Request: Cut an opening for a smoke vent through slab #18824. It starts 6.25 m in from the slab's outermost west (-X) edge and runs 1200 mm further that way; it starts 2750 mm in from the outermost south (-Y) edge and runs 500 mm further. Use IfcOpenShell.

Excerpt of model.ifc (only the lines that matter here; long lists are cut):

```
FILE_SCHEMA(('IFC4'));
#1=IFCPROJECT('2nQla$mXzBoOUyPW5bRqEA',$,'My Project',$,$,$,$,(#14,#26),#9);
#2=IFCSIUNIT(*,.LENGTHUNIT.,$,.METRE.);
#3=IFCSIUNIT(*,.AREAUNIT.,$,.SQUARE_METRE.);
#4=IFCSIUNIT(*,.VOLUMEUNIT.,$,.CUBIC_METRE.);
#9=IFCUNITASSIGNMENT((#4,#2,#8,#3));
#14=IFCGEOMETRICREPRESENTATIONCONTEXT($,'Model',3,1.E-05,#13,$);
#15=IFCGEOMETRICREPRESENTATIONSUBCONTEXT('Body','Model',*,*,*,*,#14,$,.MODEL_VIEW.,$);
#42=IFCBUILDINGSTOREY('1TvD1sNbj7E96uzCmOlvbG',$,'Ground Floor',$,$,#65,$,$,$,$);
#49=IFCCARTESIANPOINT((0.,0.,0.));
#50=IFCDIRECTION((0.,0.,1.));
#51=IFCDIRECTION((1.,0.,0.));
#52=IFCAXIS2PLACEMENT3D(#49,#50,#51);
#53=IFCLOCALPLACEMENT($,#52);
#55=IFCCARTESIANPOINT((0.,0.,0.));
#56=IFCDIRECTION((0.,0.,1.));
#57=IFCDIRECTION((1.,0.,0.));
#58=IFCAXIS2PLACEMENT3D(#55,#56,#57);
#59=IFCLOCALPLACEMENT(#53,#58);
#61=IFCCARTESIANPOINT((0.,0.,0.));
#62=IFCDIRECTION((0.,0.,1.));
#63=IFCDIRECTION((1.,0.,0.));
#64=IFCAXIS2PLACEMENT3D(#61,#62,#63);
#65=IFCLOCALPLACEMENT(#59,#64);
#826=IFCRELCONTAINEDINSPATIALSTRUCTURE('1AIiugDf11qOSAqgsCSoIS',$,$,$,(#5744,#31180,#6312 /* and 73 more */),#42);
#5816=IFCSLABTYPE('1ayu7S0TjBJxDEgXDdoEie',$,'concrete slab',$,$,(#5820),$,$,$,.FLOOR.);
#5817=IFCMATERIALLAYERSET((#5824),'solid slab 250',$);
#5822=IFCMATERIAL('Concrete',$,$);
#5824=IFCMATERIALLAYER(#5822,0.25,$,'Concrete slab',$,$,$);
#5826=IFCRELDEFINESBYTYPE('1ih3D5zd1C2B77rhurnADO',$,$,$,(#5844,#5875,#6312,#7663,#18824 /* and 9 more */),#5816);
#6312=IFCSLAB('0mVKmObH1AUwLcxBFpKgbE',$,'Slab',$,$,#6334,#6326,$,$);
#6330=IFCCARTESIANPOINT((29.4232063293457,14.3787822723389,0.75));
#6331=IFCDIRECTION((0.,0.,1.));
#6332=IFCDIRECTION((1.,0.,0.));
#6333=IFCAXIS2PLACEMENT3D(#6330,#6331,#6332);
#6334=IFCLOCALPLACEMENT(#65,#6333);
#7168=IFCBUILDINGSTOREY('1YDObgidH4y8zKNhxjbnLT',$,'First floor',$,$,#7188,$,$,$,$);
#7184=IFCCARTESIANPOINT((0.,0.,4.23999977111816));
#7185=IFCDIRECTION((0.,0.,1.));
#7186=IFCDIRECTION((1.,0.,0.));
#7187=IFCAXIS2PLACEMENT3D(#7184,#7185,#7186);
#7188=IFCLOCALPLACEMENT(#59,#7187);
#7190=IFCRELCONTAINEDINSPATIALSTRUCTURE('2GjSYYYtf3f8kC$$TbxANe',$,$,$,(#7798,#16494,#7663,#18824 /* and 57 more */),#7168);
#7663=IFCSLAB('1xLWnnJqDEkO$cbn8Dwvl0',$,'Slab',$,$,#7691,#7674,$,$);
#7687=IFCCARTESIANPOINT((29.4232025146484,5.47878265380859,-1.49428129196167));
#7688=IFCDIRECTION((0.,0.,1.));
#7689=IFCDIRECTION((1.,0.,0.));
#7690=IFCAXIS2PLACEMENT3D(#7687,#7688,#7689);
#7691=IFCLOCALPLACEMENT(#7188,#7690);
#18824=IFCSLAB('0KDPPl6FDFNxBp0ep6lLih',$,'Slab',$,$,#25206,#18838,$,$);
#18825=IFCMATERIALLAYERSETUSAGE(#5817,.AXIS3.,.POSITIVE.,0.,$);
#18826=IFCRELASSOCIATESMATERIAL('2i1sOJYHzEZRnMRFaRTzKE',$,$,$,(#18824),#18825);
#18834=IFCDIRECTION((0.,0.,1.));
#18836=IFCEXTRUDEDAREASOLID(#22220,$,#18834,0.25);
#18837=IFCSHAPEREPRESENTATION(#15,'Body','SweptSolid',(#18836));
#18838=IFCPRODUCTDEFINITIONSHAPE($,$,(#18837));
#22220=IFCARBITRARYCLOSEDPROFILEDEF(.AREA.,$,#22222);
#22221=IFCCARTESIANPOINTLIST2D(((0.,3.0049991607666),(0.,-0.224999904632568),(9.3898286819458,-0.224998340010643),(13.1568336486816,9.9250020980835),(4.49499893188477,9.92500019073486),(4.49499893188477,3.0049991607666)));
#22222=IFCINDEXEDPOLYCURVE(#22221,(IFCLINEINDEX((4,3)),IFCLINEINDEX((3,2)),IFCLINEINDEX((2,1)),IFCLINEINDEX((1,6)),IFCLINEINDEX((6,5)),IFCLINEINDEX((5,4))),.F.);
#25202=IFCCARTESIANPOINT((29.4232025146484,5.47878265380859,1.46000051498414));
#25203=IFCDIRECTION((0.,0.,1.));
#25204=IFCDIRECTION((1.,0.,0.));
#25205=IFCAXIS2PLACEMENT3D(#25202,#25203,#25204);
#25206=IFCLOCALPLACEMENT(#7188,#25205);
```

```python
import numpy as np
import ifcopenshell
import ifcopenshell.api.feature
import ifcopenshell.api.geometry
import ifcopenshell.api.root
import ifcopenshell.geom
import ifcopenshell.util.placement
import ifcopenshell.util.representation
import ifcopenshell.util.shape
import ifcopenshell.util.unit

model = ifcopenshell.open("model.ifc")
unit_scale = ifcopenshell.util.unit.calculate_unit_scale(model)
settings = ifcopenshell.geom.settings()


def volume(element):
    """Net volume in cubic metres, openings subtracted."""
    shape = ifcopenshell.geom.create_shape(settings, element)
    return ifcopenshell.util.shape.get_volume(shape.geometry)


slab = model.by_guid("0KDPPl6FDFNxBp0ep6lLih")
before = volume(slab)

# Extent in the slab's own axes, in metres. The edges named are its -X and -Y sides.
slab_shape = ifcopenshell.geom.create_shape(settings, slab)
vertices = ifcopenshell.util.shape.get_vertices(slab_shape.geometry)
x_min, y_min, bottom = vertices.min(axis=0)
top = vertices[:, 2].max()

opening = ifcopenshell.api.root.create_entity(model, ifc_class="IfcOpeningElement", name="Smoke vent opening", predefined_type="OPENING")
context = ifcopenshell.util.representation.get_context(model, "Model", "Body", "MODEL_VIEW")
width, depth = 1.2, 0.5
outline = [(0.0, 0.0), (width, 0.0), (width, depth), (0.0, depth), (0.0, 0.0)]
# Overshoot both faces by 50 mm so the cut is clean.
shape = ifcopenshell.api.geometry.add_slab_representation(
    model, context=context, depth=top - bottom + 0.1, polyline=outline
)
ifcopenshell.api.geometry.assign_representation(model, product=opening, representation=shape)

matrix = ifcopenshell.util.placement.get_local_placement(slab.ObjectPlacement)
matrix[:, 3] = matrix @ np.append(np.array([x_min + 6.25, y_min + 2.75, bottom - 0.05]) / unit_scale, 1.0)
ifcopenshell.api.geometry.edit_object_placement(model, product=opening, matrix=matrix, is_si=False)
ifcopenshell.api.feature.add_feature(model, feature=opening, element=slab)

after = volume(slab)

print(f"slab volume {before:.3f} -> {after:.3f} m3")

model.write("model-out.ifc")
```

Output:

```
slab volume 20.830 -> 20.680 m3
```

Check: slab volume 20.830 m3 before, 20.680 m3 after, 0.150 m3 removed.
